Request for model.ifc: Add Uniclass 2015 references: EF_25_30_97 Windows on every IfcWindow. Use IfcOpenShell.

First a look at what the model holds.

```python
import ifcopenshell

model = ifcopenshell.open("model.ifc")
print(model.schema)
print("classifications:", [c.Name for c in model.by_type("IfcClassification")])
for ifc_class in ("IfcDoor", "IfcRoof", "IfcStair", "IfcWall", "IfcWindow"):
    print(ifc_class, len(model.by_type(ifc_class)))
```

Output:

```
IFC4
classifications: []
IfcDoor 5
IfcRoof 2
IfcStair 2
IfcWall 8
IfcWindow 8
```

```python
import ifcopenshell
import ifcopenshell.api.classification

model = ifcopenshell.open("model.ifc")

system = ifcopenshell.api.classification.add_classification(model, classification="Uniclass 2015")

codes = {
    "IfcWindow": ("EF_25_30_97", "Windows"),
}
for ifc_class, (code, name) in codes.items():
    products = model.by_type(ifc_class)
    ifcopenshell.api.classification.add_reference(
        model, products=products, classification=system, identification=code, name=name
    )
    print(code, len(products))

model.write("model_rev.ifc")
```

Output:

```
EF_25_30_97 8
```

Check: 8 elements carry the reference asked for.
